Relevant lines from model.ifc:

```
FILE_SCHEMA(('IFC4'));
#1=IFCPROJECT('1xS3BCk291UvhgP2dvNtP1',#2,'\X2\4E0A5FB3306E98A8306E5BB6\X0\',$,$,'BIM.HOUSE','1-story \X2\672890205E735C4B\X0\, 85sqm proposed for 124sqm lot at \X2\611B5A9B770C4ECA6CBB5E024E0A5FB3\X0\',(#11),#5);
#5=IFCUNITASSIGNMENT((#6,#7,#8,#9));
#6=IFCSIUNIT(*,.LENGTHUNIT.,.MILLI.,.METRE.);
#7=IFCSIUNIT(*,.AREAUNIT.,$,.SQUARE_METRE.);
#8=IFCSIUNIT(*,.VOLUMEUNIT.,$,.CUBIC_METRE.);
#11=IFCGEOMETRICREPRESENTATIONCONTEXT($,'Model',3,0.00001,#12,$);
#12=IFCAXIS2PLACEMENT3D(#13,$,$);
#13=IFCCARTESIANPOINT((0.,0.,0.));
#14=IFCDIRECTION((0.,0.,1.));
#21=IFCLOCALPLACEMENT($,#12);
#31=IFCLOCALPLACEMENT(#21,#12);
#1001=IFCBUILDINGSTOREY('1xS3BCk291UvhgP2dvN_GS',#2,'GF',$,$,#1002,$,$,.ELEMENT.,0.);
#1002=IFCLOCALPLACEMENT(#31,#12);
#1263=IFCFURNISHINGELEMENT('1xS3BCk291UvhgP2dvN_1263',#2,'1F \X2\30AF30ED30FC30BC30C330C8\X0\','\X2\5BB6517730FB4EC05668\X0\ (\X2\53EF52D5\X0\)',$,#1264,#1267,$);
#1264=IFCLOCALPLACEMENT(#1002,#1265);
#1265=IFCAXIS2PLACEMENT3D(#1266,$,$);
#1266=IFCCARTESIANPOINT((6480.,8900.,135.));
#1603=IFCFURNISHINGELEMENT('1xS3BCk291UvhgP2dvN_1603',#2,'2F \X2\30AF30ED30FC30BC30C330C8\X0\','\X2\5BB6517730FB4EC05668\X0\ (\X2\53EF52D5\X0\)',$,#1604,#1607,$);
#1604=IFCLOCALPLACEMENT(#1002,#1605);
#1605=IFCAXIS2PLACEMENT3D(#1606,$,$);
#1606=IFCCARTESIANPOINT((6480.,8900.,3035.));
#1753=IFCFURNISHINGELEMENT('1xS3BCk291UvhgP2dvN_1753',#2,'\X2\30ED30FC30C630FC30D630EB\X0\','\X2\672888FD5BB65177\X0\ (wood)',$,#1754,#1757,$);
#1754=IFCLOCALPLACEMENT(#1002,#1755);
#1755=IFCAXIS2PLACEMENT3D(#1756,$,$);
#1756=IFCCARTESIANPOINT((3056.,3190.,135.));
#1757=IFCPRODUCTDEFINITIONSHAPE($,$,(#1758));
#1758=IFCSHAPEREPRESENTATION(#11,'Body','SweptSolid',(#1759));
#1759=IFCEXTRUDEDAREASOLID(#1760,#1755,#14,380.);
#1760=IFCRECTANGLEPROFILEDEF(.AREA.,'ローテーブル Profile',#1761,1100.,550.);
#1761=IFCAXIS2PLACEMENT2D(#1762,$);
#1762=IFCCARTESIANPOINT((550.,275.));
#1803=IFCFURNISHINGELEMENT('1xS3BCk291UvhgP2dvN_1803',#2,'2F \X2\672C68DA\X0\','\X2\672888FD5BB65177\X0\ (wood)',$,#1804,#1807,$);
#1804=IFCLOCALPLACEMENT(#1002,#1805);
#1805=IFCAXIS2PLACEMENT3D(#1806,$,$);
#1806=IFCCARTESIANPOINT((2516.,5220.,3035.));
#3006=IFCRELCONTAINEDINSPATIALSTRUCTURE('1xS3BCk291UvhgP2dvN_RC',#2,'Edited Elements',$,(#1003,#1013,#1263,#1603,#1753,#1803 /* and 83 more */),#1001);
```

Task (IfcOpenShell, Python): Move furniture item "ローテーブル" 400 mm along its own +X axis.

```python
import ifcopenshell
import ifcopenshell.api.geometry
import ifcopenshell.util.placement
import ifcopenshell.util.unit

model = ifcopenshell.open("model.ifc")
unit_scale = ifcopenshell.util.unit.calculate_unit_scale(model)

item = model.by_id(1753)
matrix = ifcopenshell.util.placement.get_local_placement(item.ObjectPlacement)
matrix[:3, 3] += matrix[:3, 0] * 0.4 / unit_scale
ifcopenshell.api.geometry.edit_object_placement(model, product=item, matrix=matrix, is_si=False)

print(ifcopenshell.util.placement.get_local_placement(item.ObjectPlacement).round(3) + 0.0)

model.write("model_updated.ifc")
```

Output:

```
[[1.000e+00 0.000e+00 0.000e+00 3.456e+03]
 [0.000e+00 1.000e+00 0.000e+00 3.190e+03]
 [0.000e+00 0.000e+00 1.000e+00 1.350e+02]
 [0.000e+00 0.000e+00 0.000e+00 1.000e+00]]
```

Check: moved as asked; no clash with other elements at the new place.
